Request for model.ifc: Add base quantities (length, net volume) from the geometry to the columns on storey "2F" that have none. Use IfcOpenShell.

First a look at what the model holds.

```python
import ifcopenshell
import ifcopenshell.util.element
import ifcopenshell.util.unit

model = ifcopenshell.open("model.ifc")
print(model.schema)
for unit_type in ("LENGTHUNIT", "AREAUNIT", "VOLUMEUNIT"):
    print(unit_type, ifcopenshell.util.unit.calculate_unit_scale(model, unit_type))
storey = next(s for s in model.by_type("IfcBuildingStorey") if s.Name == "2F")
columns = [e for e in ifcopenshell.util.element.get_decomposition(storey) if e.is_a("IfcColumn")]
for e in sorted(columns, key=lambda e: e.id()):
    print(e.id(), e.is_a(), e.Name, list(ifcopenshell.util.element.get_psets(e, qtos_only=True)), sep=" | ")
```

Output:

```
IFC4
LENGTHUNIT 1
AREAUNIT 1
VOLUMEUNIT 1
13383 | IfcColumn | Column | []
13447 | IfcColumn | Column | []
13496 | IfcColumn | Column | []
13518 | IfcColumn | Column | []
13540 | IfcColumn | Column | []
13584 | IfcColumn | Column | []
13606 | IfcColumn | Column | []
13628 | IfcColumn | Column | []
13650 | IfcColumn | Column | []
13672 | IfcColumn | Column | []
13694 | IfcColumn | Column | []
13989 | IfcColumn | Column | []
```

```python
import ifcopenshell
import ifcopenshell.api.pset
import ifcopenshell.geom
import ifcopenshell.util.element
import ifcopenshell.util.shape
import ifcopenshell.util.unit

model = ifcopenshell.open("model.ifc")
unit_scale = ifcopenshell.util.unit.calculate_unit_scale(model)
volume_scale = ifcopenshell.util.unit.calculate_unit_scale(model, "VOLUMEUNIT")
settings = ifcopenshell.geom.settings()

storey = next(s for s in model.by_type("IfcBuildingStorey") if s.Name == "2F")
columns = [e for e in ifcopenshell.util.element.get_decomposition(storey) if e.is_a("IfcColumn")]

for e in sorted(columns, key=lambda e: e.id()):
    if ifcopenshell.util.element.get_psets(e, qtos_only=True, should_inherit=False):
        continue
    # Geometry comes back in metres, in the element's own axes.
    shape = ifcopenshell.geom.create_shape(settings, e)
    values = {
        "Length": ifcopenshell.util.shape.get_z(shape.geometry) / unit_scale,
        "NetVolume": ifcopenshell.util.shape.get_volume(shape.geometry) / volume_scale,
    }
    qto = ifcopenshell.api.pset.add_qto(model, product=e, name="Qto_ColumnBaseQuantities")
    ifcopenshell.api.pset.edit_qto(model, qto=qto, properties=values)
    print(e.id(), {k: round(v, 3) for k, v in values.items()})

model.write("model_v2.ifc")
```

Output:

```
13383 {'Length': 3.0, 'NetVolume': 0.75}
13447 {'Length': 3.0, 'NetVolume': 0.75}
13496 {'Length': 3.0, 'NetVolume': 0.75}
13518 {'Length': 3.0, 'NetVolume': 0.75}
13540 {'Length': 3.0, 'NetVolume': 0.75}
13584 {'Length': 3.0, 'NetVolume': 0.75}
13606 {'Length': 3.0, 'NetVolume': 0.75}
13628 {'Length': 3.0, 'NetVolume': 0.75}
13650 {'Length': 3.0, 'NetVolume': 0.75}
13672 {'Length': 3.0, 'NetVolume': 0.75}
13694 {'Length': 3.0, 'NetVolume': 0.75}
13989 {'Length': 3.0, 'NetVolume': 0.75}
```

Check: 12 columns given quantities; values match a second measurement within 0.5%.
